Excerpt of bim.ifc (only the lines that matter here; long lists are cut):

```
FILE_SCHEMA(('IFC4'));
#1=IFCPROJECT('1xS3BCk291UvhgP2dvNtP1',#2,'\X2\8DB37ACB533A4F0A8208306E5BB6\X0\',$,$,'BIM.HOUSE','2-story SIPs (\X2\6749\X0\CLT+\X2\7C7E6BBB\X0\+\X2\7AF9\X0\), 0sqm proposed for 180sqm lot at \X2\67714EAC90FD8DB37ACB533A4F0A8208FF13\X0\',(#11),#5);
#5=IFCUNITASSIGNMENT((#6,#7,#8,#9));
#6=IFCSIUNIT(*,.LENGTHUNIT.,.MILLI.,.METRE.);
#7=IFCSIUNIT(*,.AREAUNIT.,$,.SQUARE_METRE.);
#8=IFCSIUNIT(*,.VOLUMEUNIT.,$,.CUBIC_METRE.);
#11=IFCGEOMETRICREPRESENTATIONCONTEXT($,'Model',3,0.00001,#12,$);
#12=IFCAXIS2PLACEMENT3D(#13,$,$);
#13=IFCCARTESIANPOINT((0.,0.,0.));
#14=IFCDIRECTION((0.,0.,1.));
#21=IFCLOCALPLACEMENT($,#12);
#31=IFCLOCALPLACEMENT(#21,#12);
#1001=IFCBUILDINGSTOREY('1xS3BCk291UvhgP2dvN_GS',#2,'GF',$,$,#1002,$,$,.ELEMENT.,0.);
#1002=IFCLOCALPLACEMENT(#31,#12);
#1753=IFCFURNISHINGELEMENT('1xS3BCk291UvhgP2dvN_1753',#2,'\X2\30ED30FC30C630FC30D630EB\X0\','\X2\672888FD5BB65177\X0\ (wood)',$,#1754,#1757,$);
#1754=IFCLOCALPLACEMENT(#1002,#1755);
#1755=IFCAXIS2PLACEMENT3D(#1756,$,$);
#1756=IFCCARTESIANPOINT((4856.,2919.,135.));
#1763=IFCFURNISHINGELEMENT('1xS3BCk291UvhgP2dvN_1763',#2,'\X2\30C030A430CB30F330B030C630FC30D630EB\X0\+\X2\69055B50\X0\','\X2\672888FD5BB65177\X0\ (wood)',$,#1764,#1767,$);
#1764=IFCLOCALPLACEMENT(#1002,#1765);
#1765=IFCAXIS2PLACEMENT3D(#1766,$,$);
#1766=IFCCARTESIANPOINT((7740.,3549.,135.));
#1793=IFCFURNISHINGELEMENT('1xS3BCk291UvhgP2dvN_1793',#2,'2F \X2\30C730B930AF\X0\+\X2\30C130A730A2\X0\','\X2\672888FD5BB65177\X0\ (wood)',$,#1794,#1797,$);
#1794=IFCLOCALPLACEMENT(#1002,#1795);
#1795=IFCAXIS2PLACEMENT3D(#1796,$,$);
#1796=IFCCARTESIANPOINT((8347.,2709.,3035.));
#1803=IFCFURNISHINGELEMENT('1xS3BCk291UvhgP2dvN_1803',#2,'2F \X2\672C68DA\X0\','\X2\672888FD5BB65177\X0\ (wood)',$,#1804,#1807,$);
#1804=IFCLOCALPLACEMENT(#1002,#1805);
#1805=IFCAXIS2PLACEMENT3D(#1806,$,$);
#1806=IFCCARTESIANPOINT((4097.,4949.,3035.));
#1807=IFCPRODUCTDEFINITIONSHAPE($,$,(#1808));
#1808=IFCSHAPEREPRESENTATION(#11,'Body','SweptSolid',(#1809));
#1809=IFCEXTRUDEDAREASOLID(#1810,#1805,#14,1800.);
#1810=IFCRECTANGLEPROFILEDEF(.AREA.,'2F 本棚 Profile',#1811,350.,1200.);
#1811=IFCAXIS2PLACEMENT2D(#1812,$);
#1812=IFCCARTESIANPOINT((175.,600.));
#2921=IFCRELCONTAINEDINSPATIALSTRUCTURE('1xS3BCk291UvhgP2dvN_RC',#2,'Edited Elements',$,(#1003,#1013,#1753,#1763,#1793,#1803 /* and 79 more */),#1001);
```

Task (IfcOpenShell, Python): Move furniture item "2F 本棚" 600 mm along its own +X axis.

```python
import ifcopenshell
import ifcopenshell.api.geometry
import ifcopenshell.util.placement
import ifcopenshell.util.unit

model = ifcopenshell.open("bim.ifc")
unit_scale = ifcopenshell.util.unit.calculate_unit_scale(model)

item = model.by_guid("1xS3BCk291UvhgP2dvN_1803")
matrix = ifcopenshell.util.placement.get_local_placement(item.ObjectPlacement)
matrix[:3, 3] += matrix[:3, 0] * 0.6 / unit_scale
ifcopenshell.api.geometry.edit_object_placement(model, product=item, matrix=matrix, is_si=False)

print(ifcopenshell.util.placement.get_local_placement(item.ObjectPlacement).round(3) + 0.0)

model.write("bim_updated.ifc")
```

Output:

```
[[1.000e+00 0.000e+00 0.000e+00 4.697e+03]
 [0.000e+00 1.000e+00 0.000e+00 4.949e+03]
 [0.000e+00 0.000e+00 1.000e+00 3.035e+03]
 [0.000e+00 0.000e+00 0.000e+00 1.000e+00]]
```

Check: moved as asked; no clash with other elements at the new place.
